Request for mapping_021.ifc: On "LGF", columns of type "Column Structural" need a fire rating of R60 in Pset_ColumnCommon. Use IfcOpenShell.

First a look at what the model holds.

```python
import ifcopenshell
import ifcopenshell.util.element

model = ifcopenshell.open("mapping_021.ifc")
print(model.schema)
storey = next(s for s in model.by_type("IfcBuildingStorey") if s.Name == "LGF")
columns = [e for e in ifcopenshell.util.element.get_decomposition(storey) if e.is_a("IfcColumn")]
seen = {}
for e in columns:
    element_type = ifcopenshell.util.element.get_type(e)
    key = (element_type.Name if element_type != e and element_type else None, ifcopenshell.util.element.get_pset(e, "Pset_ColumnCommon", "FireRating"))
    seen[key] = seen.get(key, 0) + 1
for (name, value), count in sorted(seen.items(), key=str):
    print(count, "x", name, "|", value)
```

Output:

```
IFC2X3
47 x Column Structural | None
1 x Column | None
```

```python
import ifcopenshell
import ifcopenshell.api.pset
import ifcopenshell.util.element

model = ifcopenshell.open("mapping_021.ifc")

storey = next(s for s in model.by_type("IfcBuildingStorey") if s.Name == "LGF")
columns = [e for e in ifcopenshell.util.element.get_decomposition(storey) if e.is_a("IfcColumn")]

count = 0
for e in columns:
    element_type = ifcopenshell.util.element.get_type(e)
    if element_type in (None, e) or element_type.Name != "Column Structural":
        continue
    # add_pset returns the element's existing set when there is one.
    pset = ifcopenshell.api.pset.add_pset(model, product=e, name="Pset_ColumnCommon")
    ifcopenshell.api.pset.edit_pset(model, pset=pset, properties={"FireRating": "R60"})
    count += 1

print(count, "columns updated")

model.write("mapping_021_updated.ifc")
```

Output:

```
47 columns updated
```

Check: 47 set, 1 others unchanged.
